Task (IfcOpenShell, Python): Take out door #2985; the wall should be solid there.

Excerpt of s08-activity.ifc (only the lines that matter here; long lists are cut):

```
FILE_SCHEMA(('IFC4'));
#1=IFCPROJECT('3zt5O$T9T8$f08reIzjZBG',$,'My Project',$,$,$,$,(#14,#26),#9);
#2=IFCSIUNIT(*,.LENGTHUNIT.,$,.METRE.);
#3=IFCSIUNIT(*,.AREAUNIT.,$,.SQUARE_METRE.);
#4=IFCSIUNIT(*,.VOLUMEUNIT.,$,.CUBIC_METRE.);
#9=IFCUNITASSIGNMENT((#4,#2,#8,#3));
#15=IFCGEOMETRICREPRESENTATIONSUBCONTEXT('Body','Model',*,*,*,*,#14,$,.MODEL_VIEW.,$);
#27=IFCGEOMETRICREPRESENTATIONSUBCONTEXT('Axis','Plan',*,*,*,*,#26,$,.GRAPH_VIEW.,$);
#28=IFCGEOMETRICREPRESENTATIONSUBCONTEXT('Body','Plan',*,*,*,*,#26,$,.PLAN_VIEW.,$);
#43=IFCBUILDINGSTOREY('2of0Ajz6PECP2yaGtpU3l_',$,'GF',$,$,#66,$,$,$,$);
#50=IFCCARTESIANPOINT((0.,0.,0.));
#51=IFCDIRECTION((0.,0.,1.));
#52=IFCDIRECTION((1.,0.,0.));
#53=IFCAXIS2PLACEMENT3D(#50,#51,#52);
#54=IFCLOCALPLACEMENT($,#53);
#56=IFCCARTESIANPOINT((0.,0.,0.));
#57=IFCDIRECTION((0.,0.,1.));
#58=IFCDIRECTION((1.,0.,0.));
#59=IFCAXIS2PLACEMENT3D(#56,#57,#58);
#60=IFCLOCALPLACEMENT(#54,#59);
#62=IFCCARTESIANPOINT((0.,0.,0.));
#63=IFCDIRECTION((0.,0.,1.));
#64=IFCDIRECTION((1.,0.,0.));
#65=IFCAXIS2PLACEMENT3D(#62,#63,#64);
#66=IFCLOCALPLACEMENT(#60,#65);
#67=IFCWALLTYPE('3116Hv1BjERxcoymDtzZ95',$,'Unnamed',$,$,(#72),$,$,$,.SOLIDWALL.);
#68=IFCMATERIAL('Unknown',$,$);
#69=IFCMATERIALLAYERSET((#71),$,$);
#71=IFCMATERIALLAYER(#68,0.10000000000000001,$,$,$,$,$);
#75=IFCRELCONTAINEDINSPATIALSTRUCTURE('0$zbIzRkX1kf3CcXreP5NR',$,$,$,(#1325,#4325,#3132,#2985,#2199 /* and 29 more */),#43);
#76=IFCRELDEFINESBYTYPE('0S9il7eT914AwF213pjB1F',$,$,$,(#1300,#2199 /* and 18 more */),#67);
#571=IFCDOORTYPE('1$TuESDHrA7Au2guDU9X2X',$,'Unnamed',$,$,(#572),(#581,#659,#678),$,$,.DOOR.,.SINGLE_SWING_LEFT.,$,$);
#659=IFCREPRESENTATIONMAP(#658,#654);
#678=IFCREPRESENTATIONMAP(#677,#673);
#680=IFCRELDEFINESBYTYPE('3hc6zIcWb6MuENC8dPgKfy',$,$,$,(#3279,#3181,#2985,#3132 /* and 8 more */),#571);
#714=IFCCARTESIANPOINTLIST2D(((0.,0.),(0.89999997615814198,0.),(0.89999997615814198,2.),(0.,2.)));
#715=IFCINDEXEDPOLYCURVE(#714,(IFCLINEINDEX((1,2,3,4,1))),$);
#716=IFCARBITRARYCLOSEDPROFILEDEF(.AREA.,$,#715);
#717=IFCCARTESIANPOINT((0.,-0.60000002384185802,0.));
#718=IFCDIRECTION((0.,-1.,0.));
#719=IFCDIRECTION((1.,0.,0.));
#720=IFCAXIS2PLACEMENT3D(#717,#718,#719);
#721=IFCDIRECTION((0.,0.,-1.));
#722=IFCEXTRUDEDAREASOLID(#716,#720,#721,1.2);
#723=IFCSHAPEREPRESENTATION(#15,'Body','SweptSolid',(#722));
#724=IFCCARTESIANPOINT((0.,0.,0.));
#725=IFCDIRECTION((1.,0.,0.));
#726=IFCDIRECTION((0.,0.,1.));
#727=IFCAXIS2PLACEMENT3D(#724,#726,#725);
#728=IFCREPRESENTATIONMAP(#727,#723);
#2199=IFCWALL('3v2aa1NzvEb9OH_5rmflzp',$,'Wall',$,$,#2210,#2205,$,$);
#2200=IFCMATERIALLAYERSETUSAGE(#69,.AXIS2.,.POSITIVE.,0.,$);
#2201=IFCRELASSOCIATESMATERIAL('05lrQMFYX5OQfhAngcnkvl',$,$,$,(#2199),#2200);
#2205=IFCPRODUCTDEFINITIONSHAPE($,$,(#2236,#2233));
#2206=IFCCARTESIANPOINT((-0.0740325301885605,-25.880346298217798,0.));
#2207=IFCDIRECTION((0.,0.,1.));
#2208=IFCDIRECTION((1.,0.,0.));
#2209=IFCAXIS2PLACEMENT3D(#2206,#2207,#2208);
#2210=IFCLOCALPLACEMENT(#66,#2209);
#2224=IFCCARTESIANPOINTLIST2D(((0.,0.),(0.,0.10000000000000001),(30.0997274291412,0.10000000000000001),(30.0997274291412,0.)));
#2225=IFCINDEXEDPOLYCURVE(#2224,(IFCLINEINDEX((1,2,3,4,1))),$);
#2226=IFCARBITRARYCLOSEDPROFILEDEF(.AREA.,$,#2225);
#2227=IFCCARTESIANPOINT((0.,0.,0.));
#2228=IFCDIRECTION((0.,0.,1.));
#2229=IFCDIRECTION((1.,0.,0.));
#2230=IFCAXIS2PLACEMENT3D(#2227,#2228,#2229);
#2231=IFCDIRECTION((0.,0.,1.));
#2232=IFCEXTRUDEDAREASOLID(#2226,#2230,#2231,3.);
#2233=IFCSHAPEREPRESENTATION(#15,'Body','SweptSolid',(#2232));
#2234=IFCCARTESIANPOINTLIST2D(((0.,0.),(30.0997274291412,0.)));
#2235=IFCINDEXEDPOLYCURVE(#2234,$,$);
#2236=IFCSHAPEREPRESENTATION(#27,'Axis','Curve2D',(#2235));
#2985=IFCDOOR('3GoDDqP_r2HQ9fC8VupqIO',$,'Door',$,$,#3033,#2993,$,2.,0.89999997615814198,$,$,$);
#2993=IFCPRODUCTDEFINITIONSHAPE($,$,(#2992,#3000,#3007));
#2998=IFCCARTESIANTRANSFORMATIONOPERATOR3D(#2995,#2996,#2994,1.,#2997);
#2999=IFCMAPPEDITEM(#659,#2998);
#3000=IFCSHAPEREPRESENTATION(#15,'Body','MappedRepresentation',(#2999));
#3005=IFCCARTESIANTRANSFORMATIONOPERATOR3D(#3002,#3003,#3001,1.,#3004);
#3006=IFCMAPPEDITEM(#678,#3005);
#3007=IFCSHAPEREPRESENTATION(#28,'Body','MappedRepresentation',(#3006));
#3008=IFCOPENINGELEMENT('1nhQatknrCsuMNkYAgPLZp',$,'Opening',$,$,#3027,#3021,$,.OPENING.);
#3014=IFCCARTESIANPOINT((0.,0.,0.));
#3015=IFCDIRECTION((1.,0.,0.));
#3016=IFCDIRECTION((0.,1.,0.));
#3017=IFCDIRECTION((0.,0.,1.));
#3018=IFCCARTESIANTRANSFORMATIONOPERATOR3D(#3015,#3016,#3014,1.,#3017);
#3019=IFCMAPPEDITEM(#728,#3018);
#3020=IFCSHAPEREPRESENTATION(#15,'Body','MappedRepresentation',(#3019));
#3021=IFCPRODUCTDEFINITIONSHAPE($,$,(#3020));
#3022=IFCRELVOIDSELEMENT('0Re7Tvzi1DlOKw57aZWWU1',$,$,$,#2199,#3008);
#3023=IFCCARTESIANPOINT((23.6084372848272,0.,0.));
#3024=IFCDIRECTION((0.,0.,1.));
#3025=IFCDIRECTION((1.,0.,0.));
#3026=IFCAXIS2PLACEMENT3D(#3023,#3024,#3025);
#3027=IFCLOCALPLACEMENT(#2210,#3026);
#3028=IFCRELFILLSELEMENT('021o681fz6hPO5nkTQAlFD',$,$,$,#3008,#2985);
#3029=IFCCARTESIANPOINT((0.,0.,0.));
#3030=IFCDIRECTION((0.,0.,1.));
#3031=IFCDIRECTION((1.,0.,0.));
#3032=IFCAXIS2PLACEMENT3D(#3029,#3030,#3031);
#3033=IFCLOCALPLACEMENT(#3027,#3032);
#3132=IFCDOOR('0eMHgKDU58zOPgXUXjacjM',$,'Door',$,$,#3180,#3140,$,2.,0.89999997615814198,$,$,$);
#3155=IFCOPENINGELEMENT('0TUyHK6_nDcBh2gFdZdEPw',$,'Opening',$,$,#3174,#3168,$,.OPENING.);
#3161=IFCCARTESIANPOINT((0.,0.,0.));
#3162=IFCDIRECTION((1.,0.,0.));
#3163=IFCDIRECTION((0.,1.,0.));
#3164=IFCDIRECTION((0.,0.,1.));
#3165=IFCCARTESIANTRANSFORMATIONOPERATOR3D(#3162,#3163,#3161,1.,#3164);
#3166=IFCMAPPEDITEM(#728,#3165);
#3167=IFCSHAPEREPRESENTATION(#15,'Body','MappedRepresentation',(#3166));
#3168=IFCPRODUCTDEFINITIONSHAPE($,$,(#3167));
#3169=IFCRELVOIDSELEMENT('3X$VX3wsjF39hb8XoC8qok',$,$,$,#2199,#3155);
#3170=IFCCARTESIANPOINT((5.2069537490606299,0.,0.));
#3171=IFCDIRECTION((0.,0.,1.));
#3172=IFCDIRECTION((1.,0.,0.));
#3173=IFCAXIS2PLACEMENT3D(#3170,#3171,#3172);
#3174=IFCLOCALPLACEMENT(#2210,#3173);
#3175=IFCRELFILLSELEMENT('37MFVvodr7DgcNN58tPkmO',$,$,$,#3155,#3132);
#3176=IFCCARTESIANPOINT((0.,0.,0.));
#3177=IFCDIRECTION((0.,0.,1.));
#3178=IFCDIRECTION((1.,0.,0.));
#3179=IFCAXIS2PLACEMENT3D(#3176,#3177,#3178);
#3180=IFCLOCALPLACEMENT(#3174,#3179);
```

```python
import ifcopenshell
import ifcopenshell.api.feature
import ifcopenshell.api.root
import ifcopenshell.geom
import ifcopenshell.util.shape

model = ifcopenshell.open("s08-activity.ifc")
settings = ifcopenshell.geom.settings()


def volume(element):
    """Net volume in cubic metres, openings subtracted."""
    shape = ifcopenshell.geom.create_shape(settings, element)
    return ifcopenshell.util.shape.get_volume(shape.geometry)


door = model.by_guid("3GoDDqP_r2HQ9fC8VupqIO")
opening = door.FillsVoids[0].RelatingOpeningElement
wall = opening.VoidsElements[0].RelatingBuildingElement
before = volume(wall)

ifcopenshell.api.root.remove_product(model, product=door)
ifcopenshell.api.feature.remove_feature(model, feature=opening)

after = volume(wall)

print(f"wall volume {before:.3f} -> {after:.3f} m3")

model.write("s08-activity_rev.ifc")
```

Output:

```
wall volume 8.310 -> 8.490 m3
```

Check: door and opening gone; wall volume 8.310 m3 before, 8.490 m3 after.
